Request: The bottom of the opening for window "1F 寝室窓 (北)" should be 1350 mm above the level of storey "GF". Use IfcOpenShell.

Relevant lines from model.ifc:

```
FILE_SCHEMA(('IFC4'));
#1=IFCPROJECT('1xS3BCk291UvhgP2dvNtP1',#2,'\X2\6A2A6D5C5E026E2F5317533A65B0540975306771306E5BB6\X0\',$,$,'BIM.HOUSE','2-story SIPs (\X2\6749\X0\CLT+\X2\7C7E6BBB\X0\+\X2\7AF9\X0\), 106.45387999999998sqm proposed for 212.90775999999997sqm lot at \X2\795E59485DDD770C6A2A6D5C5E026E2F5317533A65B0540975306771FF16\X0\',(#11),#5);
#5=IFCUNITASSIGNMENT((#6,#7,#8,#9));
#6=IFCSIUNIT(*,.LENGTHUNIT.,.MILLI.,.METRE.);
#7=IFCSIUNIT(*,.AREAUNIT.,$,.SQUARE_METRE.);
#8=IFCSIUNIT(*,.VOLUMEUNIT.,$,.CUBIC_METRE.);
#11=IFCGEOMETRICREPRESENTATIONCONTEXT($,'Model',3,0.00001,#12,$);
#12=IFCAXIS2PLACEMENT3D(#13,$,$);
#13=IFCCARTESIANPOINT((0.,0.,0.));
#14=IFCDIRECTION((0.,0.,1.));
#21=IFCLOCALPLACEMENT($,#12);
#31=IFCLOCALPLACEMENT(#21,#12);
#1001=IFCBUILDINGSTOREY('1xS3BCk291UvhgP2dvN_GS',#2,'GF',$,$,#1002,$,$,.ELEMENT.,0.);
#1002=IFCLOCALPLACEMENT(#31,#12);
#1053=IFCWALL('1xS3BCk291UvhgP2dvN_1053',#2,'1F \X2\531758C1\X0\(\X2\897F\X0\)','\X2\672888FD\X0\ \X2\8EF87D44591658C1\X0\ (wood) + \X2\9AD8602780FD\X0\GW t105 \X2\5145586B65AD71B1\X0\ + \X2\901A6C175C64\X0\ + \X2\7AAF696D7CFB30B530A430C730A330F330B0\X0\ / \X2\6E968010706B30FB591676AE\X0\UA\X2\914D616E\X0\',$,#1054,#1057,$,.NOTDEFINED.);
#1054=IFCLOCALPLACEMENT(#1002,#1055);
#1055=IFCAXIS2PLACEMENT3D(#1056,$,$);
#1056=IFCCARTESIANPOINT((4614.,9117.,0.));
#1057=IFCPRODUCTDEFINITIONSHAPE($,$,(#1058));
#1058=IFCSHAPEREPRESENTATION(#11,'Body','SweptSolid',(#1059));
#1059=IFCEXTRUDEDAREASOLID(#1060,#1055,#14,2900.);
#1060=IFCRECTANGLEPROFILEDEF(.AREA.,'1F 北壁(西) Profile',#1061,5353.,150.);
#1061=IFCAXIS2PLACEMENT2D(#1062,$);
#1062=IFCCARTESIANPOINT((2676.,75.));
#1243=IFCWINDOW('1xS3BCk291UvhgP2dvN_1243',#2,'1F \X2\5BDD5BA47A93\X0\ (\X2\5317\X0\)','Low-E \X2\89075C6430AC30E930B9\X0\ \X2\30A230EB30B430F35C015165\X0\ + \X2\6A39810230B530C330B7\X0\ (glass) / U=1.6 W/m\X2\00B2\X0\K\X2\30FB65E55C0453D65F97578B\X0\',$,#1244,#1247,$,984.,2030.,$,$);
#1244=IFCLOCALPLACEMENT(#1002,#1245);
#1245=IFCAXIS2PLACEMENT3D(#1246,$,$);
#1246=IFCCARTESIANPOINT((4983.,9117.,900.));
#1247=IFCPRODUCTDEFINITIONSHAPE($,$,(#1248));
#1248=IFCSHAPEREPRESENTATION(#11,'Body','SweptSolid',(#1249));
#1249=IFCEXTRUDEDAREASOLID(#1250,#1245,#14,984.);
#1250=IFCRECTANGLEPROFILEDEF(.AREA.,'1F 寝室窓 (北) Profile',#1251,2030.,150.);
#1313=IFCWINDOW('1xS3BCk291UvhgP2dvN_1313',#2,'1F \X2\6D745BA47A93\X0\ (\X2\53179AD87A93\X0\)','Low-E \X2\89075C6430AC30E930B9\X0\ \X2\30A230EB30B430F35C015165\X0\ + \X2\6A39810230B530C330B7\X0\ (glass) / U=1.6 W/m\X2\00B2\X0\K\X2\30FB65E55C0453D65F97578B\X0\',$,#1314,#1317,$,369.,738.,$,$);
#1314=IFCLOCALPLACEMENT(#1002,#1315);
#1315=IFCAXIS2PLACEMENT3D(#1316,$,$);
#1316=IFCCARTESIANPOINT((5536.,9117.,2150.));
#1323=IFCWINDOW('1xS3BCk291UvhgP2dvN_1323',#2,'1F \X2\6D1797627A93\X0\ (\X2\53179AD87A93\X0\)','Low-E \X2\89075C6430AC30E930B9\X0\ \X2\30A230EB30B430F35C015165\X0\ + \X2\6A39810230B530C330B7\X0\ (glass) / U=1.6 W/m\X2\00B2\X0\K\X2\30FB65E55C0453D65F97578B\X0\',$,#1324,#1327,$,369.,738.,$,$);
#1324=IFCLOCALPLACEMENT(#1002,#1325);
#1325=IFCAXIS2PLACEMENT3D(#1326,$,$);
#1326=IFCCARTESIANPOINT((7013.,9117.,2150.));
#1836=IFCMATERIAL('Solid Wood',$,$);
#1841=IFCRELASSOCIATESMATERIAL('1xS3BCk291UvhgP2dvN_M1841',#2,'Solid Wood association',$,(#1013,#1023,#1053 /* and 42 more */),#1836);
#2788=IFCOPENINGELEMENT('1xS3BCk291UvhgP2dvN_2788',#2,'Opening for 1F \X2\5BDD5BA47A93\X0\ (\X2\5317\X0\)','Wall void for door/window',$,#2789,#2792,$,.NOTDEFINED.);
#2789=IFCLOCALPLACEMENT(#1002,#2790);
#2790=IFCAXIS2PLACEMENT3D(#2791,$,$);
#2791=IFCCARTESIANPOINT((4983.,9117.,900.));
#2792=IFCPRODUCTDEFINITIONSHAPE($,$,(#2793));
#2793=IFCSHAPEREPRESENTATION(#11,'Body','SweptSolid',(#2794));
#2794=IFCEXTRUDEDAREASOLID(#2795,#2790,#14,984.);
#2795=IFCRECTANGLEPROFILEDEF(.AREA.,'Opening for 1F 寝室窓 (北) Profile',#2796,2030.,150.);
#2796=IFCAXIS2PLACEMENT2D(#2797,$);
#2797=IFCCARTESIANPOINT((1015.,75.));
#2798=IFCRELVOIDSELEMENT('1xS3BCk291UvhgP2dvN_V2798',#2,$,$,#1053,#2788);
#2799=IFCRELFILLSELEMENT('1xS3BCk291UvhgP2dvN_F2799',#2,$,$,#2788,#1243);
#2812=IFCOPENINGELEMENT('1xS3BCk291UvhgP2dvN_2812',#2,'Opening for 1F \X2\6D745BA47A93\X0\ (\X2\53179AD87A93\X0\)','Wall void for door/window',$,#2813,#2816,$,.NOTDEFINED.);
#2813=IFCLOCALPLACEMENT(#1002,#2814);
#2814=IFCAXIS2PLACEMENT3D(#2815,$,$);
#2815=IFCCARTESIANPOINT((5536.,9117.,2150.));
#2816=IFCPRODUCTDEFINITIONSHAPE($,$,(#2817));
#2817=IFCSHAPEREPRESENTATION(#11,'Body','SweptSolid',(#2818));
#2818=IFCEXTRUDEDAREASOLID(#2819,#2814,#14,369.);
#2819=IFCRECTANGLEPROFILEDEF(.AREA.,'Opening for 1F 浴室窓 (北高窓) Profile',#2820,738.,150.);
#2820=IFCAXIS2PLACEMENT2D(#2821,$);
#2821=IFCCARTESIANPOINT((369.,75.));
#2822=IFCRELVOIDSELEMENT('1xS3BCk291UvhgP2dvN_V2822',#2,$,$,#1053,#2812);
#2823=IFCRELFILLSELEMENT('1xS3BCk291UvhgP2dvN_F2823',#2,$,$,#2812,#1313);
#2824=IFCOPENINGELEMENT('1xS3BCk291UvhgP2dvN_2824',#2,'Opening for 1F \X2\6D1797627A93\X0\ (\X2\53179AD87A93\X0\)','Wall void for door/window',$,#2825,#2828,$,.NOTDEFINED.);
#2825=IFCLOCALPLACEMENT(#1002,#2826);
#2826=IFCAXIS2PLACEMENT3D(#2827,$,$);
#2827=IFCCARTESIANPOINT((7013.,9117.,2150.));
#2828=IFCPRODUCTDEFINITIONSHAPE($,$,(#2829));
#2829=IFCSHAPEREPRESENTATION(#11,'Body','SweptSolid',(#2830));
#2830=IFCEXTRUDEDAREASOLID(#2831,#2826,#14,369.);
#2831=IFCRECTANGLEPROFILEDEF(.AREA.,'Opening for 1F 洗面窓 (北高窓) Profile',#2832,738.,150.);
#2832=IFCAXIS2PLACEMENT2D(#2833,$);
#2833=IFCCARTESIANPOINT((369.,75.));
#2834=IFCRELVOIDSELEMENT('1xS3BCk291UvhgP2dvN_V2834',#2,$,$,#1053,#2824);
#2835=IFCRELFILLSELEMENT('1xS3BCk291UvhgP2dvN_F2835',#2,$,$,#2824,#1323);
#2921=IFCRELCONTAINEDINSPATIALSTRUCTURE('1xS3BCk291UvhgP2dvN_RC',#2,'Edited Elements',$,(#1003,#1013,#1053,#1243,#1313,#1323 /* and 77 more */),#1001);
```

```python
import numpy as np
import ifcopenshell
import ifcopenshell.api.geometry
import ifcopenshell.geom
import ifcopenshell.util.element
import ifcopenshell.util.placement
import ifcopenshell.util.shape
import ifcopenshell.util.unit

model = ifcopenshell.open("model.ifc")
unit_scale = ifcopenshell.util.unit.calculate_unit_scale(model)

window = model.by_guid("1xS3BCk291UvhgP2dvN_1243")
opening = window.FillsVoids[0].RelatingOpeningElement
storey = ifcopenshell.util.element.get_container(window, ifc_class="IfcBuildingStorey")
level = ifcopenshell.util.placement.get_local_placement(storey.ObjectPlacement)[2, 3]

# The opening's origin need not be at the sill, so measure its lowest point.
shape = ifcopenshell.geom.create_shape(ifcopenshell.geom.settings(), opening)
bottom = ifcopenshell.util.shape.get_shape_bottom_elevation(shape, shape.geometry) / unit_scale
dz = level + 1.35 / unit_scale - bottom

shift = np.array([0.0, 0.0, dz])
# The window is not placed relative to its opening, so move both.
for product in (opening, window):
    matrix = ifcopenshell.util.placement.get_local_placement(product.ObjectPlacement)
    matrix[:3, 3] += shift
    ifcopenshell.api.geometry.edit_object_placement(model, product=product, matrix=matrix, is_si=False)

print(f"moved by {dz * unit_scale:+.3f} m")

model.write("model_updated.ifc")
```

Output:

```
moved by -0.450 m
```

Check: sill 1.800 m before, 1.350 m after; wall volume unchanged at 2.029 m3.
